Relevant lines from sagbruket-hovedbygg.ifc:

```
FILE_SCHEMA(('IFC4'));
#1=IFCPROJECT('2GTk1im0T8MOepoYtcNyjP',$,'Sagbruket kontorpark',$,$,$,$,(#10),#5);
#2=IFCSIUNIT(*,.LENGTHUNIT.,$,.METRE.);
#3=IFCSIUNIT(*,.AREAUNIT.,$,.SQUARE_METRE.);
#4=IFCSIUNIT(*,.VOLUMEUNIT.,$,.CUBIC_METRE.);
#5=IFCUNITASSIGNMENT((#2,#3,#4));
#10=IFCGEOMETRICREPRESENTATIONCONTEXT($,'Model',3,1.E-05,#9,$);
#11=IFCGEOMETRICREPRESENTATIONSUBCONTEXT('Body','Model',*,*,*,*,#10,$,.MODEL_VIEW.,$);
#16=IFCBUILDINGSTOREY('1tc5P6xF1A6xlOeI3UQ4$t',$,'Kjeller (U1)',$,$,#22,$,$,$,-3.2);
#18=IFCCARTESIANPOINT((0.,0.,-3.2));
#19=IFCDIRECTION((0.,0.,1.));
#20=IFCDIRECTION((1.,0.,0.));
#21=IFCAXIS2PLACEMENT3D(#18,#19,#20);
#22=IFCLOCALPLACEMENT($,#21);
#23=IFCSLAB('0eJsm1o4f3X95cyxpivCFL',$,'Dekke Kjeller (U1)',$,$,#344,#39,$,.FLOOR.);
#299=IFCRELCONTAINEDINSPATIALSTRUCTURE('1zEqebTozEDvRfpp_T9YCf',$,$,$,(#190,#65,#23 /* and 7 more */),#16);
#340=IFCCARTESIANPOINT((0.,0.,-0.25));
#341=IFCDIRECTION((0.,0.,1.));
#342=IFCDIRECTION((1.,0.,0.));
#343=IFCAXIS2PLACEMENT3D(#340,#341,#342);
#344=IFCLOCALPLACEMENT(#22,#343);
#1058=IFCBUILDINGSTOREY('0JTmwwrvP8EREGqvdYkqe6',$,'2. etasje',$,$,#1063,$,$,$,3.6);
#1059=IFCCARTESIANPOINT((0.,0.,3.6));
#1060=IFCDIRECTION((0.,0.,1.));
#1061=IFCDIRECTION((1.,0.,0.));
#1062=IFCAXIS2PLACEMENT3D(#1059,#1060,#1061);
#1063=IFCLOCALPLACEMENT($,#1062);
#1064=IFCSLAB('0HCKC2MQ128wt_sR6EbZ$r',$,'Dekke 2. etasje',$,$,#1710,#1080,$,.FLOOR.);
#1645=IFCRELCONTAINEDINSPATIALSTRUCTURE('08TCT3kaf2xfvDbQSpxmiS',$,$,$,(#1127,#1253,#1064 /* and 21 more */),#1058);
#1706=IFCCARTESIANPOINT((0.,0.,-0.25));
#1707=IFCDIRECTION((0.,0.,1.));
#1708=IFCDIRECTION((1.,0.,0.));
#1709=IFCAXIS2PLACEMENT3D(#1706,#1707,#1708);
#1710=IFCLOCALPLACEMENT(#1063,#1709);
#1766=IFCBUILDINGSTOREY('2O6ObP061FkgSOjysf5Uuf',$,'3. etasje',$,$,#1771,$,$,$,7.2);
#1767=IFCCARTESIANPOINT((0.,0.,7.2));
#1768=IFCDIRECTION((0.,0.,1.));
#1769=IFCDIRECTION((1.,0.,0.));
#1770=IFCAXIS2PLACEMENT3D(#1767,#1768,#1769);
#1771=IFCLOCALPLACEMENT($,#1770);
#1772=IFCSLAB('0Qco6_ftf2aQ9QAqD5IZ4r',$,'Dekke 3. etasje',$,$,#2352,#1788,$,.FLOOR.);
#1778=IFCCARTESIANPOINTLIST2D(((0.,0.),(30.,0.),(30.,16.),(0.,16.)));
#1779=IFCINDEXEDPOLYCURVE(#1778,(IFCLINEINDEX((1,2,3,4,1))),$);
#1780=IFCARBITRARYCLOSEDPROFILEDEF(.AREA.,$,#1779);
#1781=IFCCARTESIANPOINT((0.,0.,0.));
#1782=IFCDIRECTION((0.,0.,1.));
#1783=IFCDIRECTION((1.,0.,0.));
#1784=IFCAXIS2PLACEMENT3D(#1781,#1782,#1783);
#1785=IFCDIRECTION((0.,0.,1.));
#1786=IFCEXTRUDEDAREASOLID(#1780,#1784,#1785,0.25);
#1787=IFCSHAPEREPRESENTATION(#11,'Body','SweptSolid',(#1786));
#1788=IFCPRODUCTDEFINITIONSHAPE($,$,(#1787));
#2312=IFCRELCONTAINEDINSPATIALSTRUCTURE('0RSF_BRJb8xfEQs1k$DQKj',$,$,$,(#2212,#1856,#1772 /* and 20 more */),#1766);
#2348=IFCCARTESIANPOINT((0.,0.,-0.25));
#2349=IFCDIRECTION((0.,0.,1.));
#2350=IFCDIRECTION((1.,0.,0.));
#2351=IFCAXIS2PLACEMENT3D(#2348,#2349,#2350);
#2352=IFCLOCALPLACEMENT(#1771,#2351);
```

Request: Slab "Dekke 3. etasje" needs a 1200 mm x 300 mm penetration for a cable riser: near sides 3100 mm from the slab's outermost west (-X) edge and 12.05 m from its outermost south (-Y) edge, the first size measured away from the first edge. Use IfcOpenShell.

```python
import numpy as np
import ifcopenshell
import ifcopenshell.api.feature
import ifcopenshell.api.geometry
import ifcopenshell.api.root
import ifcopenshell.geom
import ifcopenshell.util.placement
import ifcopenshell.util.representation
import ifcopenshell.util.shape
import ifcopenshell.util.unit

model = ifcopenshell.open("sagbruket-hovedbygg.ifc")
unit_scale = ifcopenshell.util.unit.calculate_unit_scale(model)
settings = ifcopenshell.geom.settings()


def volume(element):
    """Net volume in cubic metres, openings subtracted."""
    shape = ifcopenshell.geom.create_shape(settings, element)
    return ifcopenshell.util.shape.get_volume(shape.geometry)


slab = model.by_guid("0Qco6_ftf2aQ9QAqD5IZ4r")
before = volume(slab)

# Extent in the slab's own axes, in metres. The edges named are its -X and -Y sides.
slab_shape = ifcopenshell.geom.create_shape(settings, slab)
vertices = ifcopenshell.util.shape.get_vertices(slab_shape.geometry)
x_min, y_min, bottom = vertices.min(axis=0)
top = vertices[:, 2].max()

opening = ifcopenshell.api.root.create_entity(model, ifc_class="IfcOpeningElement", name="Cable riser opening", predefined_type="OPENING")
context = ifcopenshell.util.representation.get_context(model, "Model", "Body", "MODEL_VIEW")
width, depth = 1.2, 0.3
outline = [(0.0, 0.0), (width, 0.0), (width, depth), (0.0, depth), (0.0, 0.0)]
# Overshoot both faces by 50 mm so the cut is clean.
shape = ifcopenshell.api.geometry.add_slab_representation(
    model, context=context, depth=top - bottom + 0.1, polyline=outline
)
ifcopenshell.api.geometry.assign_representation(model, product=opening, representation=shape)

matrix = ifcopenshell.util.placement.get_local_placement(slab.ObjectPlacement)
matrix[:, 3] = matrix @ np.append(np.array([x_min + 3.1, y_min + 12.05, bottom - 0.05]) / unit_scale, 1.0)
ifcopenshell.api.geometry.edit_object_placement(model, product=opening, matrix=matrix, is_si=False)
ifcopenshell.api.feature.add_feature(model, feature=opening, element=slab)

after = volume(slab)

print(f"slab volume {before:.3f} -> {after:.3f} m3")

model.write("sagbruket-hovedbygg_edited.ifc")
```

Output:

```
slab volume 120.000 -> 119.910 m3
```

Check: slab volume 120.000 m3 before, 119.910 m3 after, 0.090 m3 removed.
